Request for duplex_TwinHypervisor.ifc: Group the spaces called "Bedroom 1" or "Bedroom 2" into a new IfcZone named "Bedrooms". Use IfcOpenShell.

First a look at what the model holds.

```python
import ifcopenshell

model = ifcopenshell.open("duplex_TwinHypervisor.ifc")
print(model.schema)
seen = {}
for space in model.by_type("IfcSpace"):
    seen[space.LongName] = seen.get(space.LongName, 0) + 1
for name, count in sorted(seen.items(), key=str):
    print(count, "x", name)
print("zones:", [z.Name for z in model.by_type("IfcZone")][:20])
```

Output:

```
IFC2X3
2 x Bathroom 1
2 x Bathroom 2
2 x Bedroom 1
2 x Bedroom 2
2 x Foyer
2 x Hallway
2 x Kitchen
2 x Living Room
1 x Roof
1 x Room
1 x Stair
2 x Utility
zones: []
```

```python
import ifcopenshell
import ifcopenshell.api.group
import ifcopenshell.api.root

model = ifcopenshell.open("duplex_TwinHypervisor.ifc")

names = {"Bedroom 1", "Bedroom 2"}
spaces = [s for s in model.by_type("IfcSpace") if s.LongName in names]

zone = ifcopenshell.api.root.create_entity(model, ifc_class="IfcZone", name="Bedrooms")
ifcopenshell.api.group.assign_group(model, products=spaces, group=zone)
print(len(spaces), "spaces in", zone.Name)

model.write("duplex_TwinHypervisor_edited.ifc")
```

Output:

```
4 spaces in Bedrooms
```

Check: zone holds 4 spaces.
